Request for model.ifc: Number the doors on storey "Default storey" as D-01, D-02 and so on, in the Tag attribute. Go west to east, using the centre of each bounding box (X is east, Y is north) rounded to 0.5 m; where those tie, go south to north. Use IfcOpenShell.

First a look at what the model holds.

```python
import ifcopenshell
import ifcopenshell.util.element
import ifcopenshell.util.placement

model = ifcopenshell.open("model.ifc")
print(model.schema)
storey = next(s for s in model.by_type("IfcBuildingStorey") if s.Name == "Default storey")
doors = [e for e in ifcopenshell.util.element.get_decomposition(storey) if e.is_a("IfcDoor")]
for e in sorted(doors, key=lambda e: e.id()):
    origin = ifcopenshell.util.placement.get_local_placement(e.ObjectPlacement)[:3, 3]
    print(e.id(), e.Tag, e.Name, origin.round(2) + 0.0, sep=" | ")
```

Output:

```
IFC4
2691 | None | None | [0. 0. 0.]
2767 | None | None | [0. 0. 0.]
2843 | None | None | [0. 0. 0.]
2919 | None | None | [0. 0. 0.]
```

```python
import ifcopenshell
import ifcopenshell.geom
import ifcopenshell.util.element
import ifcopenshell.util.shape

model = ifcopenshell.open("model.ifc")
settings = ifcopenshell.geom.settings()
settings.set("use-world-coords", True)


def centre(element):
    shape = ifcopenshell.geom.create_shape(settings, element)
    return ifcopenshell.util.shape.get_bbox_centroid(shape.geometry)


storey = next(s for s in model.by_type("IfcBuildingStorey") if s.Name == "Default storey")
doors = [e for e in ifcopenshell.util.element.get_decomposition(storey) if e.is_a("IfcDoor")]

# Insertion points can sit at a corner or the storey origin, so sort by the geometry (in metres).
centres = {e: centre(e) for e in doors}
doors.sort(key=lambda e: (round(centres[e][0] / 0.5), centres[e][1]))

for i, e in enumerate(doors, start=1):
    number = f"D-{i:02d}"
    e.Tag = number
    print(e.id(), number)

model.write("model-out.ifc")
```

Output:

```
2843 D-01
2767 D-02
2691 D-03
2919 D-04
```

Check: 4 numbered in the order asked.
